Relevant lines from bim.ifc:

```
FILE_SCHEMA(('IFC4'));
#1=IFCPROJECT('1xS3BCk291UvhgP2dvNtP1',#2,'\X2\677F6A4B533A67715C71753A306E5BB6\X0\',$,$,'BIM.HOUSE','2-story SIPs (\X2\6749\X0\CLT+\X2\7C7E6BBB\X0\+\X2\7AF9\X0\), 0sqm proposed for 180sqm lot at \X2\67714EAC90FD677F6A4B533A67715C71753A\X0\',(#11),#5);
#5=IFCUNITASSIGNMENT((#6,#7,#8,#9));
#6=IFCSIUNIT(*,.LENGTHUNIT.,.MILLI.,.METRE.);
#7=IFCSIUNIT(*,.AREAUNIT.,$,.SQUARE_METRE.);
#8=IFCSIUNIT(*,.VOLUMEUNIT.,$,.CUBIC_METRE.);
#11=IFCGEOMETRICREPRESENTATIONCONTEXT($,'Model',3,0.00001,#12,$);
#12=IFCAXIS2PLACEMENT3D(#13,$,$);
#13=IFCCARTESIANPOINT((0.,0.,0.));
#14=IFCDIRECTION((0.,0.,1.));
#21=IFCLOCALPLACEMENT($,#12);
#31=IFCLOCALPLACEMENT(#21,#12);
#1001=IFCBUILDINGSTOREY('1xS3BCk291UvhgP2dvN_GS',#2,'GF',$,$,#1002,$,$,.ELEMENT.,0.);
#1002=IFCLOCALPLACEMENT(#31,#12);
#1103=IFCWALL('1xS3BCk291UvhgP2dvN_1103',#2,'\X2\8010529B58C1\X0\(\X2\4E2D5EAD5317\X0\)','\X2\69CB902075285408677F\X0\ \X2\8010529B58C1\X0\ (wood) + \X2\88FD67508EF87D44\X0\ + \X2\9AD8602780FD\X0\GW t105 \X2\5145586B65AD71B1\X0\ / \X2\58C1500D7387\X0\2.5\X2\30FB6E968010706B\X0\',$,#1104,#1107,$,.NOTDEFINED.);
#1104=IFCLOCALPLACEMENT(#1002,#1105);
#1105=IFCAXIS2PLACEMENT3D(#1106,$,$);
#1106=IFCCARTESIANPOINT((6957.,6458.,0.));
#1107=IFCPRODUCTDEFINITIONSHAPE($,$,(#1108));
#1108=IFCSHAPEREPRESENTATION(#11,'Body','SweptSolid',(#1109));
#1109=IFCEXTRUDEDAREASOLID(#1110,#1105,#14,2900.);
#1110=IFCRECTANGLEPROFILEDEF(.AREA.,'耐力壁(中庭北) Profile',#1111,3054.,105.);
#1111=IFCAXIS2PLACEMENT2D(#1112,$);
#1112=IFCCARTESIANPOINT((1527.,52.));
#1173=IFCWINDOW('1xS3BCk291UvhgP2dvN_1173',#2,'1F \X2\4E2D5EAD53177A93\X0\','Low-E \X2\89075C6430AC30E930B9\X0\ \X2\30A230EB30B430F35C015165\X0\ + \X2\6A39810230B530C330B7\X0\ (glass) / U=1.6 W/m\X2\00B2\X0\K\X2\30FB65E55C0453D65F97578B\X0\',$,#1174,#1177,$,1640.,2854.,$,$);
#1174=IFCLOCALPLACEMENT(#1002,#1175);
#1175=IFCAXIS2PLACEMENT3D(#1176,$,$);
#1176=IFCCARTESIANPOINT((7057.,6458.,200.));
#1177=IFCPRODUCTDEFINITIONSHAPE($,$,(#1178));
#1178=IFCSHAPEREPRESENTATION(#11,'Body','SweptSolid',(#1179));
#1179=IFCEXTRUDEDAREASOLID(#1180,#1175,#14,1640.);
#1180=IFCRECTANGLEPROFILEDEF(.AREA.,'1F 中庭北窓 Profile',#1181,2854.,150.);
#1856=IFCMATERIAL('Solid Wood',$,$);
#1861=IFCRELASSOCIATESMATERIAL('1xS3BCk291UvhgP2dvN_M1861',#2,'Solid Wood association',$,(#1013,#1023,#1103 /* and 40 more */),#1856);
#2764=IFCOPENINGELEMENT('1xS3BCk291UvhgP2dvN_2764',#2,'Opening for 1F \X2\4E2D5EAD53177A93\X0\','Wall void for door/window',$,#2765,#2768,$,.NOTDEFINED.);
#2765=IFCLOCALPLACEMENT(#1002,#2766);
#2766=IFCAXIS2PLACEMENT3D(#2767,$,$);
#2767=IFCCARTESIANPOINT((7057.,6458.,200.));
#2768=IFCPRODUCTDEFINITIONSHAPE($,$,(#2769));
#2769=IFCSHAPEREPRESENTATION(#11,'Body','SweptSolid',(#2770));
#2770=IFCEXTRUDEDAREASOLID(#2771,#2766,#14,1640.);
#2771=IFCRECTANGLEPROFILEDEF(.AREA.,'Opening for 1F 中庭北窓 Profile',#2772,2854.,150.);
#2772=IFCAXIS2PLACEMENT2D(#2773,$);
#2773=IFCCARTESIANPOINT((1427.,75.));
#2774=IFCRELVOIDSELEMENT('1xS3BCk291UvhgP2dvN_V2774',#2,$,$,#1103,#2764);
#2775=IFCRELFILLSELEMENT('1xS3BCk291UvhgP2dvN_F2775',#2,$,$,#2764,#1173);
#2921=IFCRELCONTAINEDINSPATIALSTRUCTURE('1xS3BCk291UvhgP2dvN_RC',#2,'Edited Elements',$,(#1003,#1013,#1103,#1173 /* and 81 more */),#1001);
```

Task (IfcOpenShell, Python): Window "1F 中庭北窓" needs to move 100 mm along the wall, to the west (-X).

```python
import ifcopenshell
import ifcopenshell.api.geometry
import ifcopenshell.util.placement
import ifcopenshell.util.unit

model = ifcopenshell.open("bim.ifc")
unit_scale = ifcopenshell.util.unit.calculate_unit_scale(model)

window = model.by_id(1173)
opening = window.FillsVoids[0].RelatingOpeningElement
wall = opening.VoidsElements[0].RelatingBuildingElement

wall_matrix = ifcopenshell.util.placement.get_local_placement(wall.ObjectPlacement)
shift = wall_matrix[:3, 0] * -0.1 / unit_scale
before = ifcopenshell.util.placement.get_local_placement(window.ObjectPlacement)[:3, 3].copy()

# The window is not placed relative to its opening, so move both.
for product in (opening, window):
    matrix = ifcopenshell.util.placement.get_local_placement(product.ObjectPlacement)
    matrix[:3, 3] += shift
    ifcopenshell.api.geometry.edit_object_placement(model, product=product, matrix=matrix, is_si=False)

after = ifcopenshell.util.placement.get_local_placement(window.ObjectPlacement)[:3, 3]
print("window moved by", (after - before).round(3) + 0.0)

model.write("bim_updated.ifc")
```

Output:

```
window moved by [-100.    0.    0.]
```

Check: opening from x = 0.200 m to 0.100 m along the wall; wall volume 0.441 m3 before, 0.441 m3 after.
